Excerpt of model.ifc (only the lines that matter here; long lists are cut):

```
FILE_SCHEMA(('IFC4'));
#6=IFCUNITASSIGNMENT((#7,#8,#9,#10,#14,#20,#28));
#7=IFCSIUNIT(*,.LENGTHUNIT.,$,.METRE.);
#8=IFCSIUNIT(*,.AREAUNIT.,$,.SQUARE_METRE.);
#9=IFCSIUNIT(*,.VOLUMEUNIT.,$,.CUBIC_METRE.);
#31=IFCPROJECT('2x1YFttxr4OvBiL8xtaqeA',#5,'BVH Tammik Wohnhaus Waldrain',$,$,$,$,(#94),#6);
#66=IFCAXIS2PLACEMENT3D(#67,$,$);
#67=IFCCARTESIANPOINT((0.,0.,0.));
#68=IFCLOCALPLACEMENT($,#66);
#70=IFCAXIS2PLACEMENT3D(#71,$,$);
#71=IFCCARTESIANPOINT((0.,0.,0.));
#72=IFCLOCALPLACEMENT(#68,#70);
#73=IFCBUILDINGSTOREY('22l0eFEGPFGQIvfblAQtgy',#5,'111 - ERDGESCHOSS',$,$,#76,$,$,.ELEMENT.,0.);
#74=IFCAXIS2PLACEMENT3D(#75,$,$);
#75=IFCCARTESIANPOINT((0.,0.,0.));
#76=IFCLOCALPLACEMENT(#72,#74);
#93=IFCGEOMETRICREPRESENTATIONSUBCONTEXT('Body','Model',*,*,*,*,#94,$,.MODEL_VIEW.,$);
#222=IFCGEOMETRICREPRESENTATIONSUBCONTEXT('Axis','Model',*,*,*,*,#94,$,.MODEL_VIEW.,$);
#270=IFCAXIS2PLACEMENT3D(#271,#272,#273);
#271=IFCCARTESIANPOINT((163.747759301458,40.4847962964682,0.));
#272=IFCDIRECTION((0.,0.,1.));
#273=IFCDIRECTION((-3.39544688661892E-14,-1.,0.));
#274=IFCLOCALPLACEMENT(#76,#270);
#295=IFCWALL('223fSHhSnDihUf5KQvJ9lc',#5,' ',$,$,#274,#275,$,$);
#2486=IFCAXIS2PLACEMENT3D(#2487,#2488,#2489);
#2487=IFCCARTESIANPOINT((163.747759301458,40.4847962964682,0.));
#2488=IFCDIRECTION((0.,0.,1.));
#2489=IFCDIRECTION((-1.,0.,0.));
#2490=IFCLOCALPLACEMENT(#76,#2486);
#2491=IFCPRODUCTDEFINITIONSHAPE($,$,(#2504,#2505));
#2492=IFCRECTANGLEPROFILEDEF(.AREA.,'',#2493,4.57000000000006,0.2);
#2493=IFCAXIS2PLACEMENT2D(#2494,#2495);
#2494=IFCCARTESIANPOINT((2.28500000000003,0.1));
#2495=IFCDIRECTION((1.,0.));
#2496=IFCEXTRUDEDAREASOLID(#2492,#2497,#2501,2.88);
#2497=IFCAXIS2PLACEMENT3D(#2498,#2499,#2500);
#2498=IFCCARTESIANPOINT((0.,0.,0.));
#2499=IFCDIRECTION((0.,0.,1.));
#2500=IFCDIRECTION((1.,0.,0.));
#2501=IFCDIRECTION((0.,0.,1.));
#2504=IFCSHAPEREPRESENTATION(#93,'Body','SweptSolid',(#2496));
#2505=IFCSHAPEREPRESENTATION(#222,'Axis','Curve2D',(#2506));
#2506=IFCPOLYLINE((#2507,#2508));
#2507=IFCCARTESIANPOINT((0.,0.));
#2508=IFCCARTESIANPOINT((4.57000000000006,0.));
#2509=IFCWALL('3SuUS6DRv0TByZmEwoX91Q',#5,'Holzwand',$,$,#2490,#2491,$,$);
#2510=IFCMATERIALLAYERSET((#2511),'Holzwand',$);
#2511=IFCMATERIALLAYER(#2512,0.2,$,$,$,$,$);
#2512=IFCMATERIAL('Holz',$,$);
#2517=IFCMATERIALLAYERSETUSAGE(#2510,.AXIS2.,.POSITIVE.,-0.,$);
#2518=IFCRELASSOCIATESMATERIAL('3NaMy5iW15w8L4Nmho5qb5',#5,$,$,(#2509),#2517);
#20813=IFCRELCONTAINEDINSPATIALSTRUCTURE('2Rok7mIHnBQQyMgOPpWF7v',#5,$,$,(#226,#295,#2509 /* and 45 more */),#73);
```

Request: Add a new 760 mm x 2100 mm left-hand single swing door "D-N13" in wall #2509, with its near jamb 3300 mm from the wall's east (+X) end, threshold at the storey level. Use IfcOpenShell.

```python
import numpy as np
import ifcopenshell
import ifcopenshell.api.feature
import ifcopenshell.api.geometry
import ifcopenshell.api.root
import ifcopenshell.api.spatial
import ifcopenshell.geom
import ifcopenshell.util.element
import ifcopenshell.util.placement
import ifcopenshell.util.representation
import ifcopenshell.util.shape
import ifcopenshell.util.unit

model = ifcopenshell.open("model.ifc")
unit_scale = ifcopenshell.util.unit.calculate_unit_scale(model)
settings = ifcopenshell.geom.settings()


def volume(element):
    """Net volume in cubic metres, openings subtracted."""
    shape = ifcopenshell.geom.create_shape(settings, element)
    return ifcopenshell.util.shape.get_volume(shape.geometry)


wall = model.by_id(2509)
storey = ifcopenshell.util.element.get_container(wall, ifc_class="IfcBuildingStorey")
context = ifcopenshell.util.representation.get_context(model, "Model", "Body", "MODEL_VIEW")
before = volume(wall)

width, height, from_end, sill = 0.76, 2.1, 3.3, 0.0  # metres

# The wall runs along its own X axis, and the end named is its -X end.
wall_shape = ifcopenshell.geom.create_shape(settings, wall)
x, y, z = ifcopenshell.util.shape.get_vertices(wall_shape.geometry).T
start = x.min() + from_end
face, thickness = float(y.min()), float(y.max() - y.min())
wall_matrix = ifcopenshell.util.placement.get_local_placement(wall.ObjectPlacement)
level = ifcopenshell.util.placement.get_local_placement(storey.ObjectPlacement)[2, 3]


def in_wall(x, y):
    """Placement at x, y metres in the wall's axes, at sill height."""
    matrix = wall_matrix.copy()
    matrix[:, 3] = wall_matrix @ np.array([x / unit_scale, y / unit_scale, 0.0, 1.0])
    matrix[2, 3] = level + sill / unit_scale
    return matrix


# Opening: a box that overshoots both wall faces by 50 mm.
opening = ifcopenshell.api.root.create_entity(model, ifc_class="IfcOpeningElement", predefined_type="OPENING")
box = ifcopenshell.api.geometry.add_wall_representation(
    model, context=context, length=width, height=height, thickness=thickness + 0.1
)
ifcopenshell.api.geometry.assign_representation(model, product=opening, representation=box)
ifcopenshell.api.geometry.edit_object_placement(model, product=opening, matrix=in_wall(start, face - 0.05), is_si=False)
ifcopenshell.api.feature.add_feature(model, feature=opening, element=wall)

door = ifcopenshell.api.root.create_entity(model, ifc_class="IfcDoor", name="D-N13", predefined_type="DOOR")
door.OverallWidth, door.OverallHeight = width / unit_scale, height / unit_scale
door.OperationType = "SINGLE_SWING_LEFT"
body = ifcopenshell.api.geometry.add_door_representation(
    model,
    context=context,
    overall_width=door.OverallWidth,
    overall_height=door.OverallHeight,
    operation_type="SINGLE_SWING_LEFT",
    lining_properties={"LiningDepth": thickness / unit_scale, "ThresholdDepth": thickness / unit_scale},
)
ifcopenshell.api.geometry.assign_representation(model, product=door, representation=body)
ifcopenshell.api.spatial.assign_container(model, products=[door], relating_structure=storey)
ifcopenshell.api.feature.add_filling(model, opening=opening, element=door)

# The lining spans the wall, so the door starts at the wall face.
ifcopenshell.api.geometry.edit_object_placement(model, product=door, matrix=in_wall(start, face), is_si=False)

after = volume(wall)

print(f"wall volume {before:.3f} -> {after:.3f} m3")

model.write("model-out.ifc")
```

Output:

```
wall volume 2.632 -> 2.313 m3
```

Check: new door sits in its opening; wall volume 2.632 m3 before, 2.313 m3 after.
